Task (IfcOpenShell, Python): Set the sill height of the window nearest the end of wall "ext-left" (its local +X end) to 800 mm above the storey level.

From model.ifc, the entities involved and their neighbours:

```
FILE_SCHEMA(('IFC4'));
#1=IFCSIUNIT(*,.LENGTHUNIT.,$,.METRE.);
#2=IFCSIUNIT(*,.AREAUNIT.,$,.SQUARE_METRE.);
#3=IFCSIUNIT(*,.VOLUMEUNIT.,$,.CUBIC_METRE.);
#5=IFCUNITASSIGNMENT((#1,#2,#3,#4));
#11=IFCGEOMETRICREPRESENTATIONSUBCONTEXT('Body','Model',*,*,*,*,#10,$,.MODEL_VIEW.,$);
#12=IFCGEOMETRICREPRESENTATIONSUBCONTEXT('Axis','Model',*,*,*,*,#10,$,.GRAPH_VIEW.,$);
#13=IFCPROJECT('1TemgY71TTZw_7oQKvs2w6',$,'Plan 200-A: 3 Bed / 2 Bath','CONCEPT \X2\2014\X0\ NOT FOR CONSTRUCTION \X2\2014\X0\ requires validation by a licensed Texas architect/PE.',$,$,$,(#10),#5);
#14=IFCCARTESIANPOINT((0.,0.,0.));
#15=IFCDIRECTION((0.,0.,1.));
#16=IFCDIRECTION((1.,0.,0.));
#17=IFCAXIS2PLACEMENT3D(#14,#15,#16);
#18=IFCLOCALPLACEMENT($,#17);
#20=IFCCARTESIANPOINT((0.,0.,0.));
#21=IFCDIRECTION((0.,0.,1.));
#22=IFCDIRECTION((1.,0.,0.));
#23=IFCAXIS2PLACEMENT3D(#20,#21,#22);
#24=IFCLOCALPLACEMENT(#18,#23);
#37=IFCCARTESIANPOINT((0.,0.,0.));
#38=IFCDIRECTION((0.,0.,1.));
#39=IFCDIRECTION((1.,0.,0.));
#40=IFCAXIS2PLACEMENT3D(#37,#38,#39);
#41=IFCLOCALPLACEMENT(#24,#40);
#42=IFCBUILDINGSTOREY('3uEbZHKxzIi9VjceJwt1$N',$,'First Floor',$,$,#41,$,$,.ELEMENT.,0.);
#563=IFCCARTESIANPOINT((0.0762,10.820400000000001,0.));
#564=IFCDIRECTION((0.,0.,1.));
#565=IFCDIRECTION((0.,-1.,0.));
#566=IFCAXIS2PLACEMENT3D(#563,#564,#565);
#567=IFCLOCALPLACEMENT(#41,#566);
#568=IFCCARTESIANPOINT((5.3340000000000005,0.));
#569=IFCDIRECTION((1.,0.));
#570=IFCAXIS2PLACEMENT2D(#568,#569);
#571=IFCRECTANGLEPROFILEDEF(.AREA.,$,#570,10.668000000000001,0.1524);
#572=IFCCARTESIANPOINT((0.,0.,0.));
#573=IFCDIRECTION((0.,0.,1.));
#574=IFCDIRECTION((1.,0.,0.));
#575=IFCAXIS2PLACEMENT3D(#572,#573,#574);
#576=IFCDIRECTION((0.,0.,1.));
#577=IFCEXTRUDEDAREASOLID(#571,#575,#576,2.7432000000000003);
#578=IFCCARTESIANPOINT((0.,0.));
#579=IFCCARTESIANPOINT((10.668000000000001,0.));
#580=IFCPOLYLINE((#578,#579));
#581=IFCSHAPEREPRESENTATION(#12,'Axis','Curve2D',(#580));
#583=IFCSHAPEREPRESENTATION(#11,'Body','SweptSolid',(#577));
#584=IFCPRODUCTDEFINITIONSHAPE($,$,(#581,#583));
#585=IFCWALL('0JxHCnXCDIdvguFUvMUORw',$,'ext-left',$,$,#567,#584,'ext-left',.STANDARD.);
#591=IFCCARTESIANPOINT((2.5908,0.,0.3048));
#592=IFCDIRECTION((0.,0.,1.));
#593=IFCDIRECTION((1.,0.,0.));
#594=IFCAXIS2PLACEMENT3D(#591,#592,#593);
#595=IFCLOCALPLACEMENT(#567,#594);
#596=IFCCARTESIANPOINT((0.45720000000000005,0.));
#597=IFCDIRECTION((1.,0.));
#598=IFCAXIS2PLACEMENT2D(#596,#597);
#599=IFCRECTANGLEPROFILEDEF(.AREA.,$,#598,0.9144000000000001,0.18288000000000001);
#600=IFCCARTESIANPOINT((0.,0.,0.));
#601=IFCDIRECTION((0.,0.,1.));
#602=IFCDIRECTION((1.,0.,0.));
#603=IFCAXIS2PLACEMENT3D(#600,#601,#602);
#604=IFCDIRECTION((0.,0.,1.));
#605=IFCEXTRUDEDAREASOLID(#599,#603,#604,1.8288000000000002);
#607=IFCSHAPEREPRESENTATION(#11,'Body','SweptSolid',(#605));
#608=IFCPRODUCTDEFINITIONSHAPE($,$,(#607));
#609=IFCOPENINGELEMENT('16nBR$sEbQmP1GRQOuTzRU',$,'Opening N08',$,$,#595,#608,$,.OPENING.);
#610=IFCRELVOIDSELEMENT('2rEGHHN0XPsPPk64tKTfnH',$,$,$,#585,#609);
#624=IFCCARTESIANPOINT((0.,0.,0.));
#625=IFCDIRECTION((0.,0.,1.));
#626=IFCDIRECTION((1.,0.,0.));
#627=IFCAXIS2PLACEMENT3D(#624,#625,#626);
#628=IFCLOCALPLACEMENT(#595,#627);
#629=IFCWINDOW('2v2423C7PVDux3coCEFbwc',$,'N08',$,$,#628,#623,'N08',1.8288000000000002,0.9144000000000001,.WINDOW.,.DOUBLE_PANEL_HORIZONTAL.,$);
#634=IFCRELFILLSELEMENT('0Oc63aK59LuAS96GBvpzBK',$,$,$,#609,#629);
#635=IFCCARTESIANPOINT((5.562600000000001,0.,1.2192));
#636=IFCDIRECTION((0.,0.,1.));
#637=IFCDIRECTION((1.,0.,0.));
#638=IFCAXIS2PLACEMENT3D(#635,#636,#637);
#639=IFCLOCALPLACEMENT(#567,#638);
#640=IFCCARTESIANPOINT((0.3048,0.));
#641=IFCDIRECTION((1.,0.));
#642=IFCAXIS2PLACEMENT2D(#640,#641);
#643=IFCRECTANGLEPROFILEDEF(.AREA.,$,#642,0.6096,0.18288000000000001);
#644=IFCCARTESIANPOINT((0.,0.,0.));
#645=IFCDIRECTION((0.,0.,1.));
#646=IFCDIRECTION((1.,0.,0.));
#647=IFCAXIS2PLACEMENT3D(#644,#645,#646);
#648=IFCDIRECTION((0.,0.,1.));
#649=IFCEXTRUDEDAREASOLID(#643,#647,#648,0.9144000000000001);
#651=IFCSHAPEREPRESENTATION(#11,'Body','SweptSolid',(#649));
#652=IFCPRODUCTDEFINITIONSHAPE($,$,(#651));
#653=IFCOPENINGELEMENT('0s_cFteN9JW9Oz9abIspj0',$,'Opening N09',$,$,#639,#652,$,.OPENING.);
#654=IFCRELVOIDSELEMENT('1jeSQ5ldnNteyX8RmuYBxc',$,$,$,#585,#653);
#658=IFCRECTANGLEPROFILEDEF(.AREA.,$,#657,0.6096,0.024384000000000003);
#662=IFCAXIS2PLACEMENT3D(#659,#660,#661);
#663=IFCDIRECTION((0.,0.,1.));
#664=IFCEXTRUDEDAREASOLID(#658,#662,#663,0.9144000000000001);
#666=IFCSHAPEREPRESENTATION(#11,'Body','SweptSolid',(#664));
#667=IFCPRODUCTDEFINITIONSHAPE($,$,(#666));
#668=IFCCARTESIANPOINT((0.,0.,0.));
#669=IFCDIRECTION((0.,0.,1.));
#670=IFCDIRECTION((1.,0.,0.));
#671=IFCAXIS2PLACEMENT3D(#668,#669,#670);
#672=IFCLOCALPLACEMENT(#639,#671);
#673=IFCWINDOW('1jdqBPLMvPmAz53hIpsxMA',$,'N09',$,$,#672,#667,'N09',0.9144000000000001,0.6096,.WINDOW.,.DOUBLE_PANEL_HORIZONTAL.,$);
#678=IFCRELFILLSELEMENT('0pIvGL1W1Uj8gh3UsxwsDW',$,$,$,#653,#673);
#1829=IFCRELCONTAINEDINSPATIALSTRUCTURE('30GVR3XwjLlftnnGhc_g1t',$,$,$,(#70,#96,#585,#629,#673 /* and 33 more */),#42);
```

```python
import numpy as np
import ifcopenshell
import ifcopenshell.api.geometry
import ifcopenshell.geom
import ifcopenshell.util.element
import ifcopenshell.util.placement
import ifcopenshell.util.shape
import ifcopenshell.util.unit

model = ifcopenshell.open("model.ifc")
unit_scale = ifcopenshell.util.unit.calculate_unit_scale(model)

window = model.by_guid("1jdqBPLMvPmAz53hIpsxMA")
opening = window.FillsVoids[0].RelatingOpeningElement
storey = ifcopenshell.util.element.get_container(window, ifc_class="IfcBuildingStorey")
level = ifcopenshell.util.placement.get_local_placement(storey.ObjectPlacement)[2, 3]

# The opening's origin need not be at the sill, so measure its lowest point.
shape = ifcopenshell.geom.create_shape(ifcopenshell.geom.settings(), opening)
bottom = ifcopenshell.util.shape.get_shape_bottom_elevation(shape, shape.geometry) / unit_scale
dz = level + 0.8 - bottom

shift = np.array([0.0, 0.0, dz])
# The window is placed relative to its opening, so it follows when the opening moves.
matrix = ifcopenshell.util.placement.get_local_placement(opening.ObjectPlacement)
matrix[:3, 3] += shift
ifcopenshell.api.geometry.edit_object_placement(
    model, product=opening, matrix=matrix, is_si=False, should_transform_children=True
)

print(f"moved by {dz * unit_scale:+.3f} m")

model.write("model-out.ifc")
```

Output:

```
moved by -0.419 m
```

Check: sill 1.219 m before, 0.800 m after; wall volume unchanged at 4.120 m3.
